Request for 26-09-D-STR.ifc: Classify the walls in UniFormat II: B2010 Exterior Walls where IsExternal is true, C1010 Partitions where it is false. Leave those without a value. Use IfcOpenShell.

First a look at what the model holds.

```python
import ifcopenshell
import ifcopenshell.util.element

model = ifcopenshell.open("26-09-D-STR.ifc")
print(model.schema)
print("classifications:", [c.Name for c in model.by_type("IfcClassification")])
values = [ifcopenshell.util.element.get_pset(e, "Pset_WallCommon", "IsExternal") for e in model.by_type("IfcWall")]
for value in (True, False, None):
    print("IsExternal", value, values.count(value))
```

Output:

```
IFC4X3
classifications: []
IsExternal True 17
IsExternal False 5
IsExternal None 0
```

```python
import ifcopenshell
import ifcopenshell.api.classification
import ifcopenshell.util.element

model = ifcopenshell.open("26-09-D-STR.ifc")

system = ifcopenshell.api.classification.add_classification(model, classification="UniFormat II")

walls = model.by_type("IfcWall")
external = {e: ifcopenshell.util.element.get_pset(e, "Pset_WallCommon", "IsExternal") for e in walls}
for flag, code, name in ((True, "B2010", "Exterior Walls"), (False, "C1010", "Partitions")):
    products = [e for e in walls if external[e] is flag]
    ifcopenshell.api.classification.add_reference(
        model, products=products, classification=system, identification=code, name=name
    )
    print(code, len(products))

model.write("26-09-D-STR_v2.ifc")
```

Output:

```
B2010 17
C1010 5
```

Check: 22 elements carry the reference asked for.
